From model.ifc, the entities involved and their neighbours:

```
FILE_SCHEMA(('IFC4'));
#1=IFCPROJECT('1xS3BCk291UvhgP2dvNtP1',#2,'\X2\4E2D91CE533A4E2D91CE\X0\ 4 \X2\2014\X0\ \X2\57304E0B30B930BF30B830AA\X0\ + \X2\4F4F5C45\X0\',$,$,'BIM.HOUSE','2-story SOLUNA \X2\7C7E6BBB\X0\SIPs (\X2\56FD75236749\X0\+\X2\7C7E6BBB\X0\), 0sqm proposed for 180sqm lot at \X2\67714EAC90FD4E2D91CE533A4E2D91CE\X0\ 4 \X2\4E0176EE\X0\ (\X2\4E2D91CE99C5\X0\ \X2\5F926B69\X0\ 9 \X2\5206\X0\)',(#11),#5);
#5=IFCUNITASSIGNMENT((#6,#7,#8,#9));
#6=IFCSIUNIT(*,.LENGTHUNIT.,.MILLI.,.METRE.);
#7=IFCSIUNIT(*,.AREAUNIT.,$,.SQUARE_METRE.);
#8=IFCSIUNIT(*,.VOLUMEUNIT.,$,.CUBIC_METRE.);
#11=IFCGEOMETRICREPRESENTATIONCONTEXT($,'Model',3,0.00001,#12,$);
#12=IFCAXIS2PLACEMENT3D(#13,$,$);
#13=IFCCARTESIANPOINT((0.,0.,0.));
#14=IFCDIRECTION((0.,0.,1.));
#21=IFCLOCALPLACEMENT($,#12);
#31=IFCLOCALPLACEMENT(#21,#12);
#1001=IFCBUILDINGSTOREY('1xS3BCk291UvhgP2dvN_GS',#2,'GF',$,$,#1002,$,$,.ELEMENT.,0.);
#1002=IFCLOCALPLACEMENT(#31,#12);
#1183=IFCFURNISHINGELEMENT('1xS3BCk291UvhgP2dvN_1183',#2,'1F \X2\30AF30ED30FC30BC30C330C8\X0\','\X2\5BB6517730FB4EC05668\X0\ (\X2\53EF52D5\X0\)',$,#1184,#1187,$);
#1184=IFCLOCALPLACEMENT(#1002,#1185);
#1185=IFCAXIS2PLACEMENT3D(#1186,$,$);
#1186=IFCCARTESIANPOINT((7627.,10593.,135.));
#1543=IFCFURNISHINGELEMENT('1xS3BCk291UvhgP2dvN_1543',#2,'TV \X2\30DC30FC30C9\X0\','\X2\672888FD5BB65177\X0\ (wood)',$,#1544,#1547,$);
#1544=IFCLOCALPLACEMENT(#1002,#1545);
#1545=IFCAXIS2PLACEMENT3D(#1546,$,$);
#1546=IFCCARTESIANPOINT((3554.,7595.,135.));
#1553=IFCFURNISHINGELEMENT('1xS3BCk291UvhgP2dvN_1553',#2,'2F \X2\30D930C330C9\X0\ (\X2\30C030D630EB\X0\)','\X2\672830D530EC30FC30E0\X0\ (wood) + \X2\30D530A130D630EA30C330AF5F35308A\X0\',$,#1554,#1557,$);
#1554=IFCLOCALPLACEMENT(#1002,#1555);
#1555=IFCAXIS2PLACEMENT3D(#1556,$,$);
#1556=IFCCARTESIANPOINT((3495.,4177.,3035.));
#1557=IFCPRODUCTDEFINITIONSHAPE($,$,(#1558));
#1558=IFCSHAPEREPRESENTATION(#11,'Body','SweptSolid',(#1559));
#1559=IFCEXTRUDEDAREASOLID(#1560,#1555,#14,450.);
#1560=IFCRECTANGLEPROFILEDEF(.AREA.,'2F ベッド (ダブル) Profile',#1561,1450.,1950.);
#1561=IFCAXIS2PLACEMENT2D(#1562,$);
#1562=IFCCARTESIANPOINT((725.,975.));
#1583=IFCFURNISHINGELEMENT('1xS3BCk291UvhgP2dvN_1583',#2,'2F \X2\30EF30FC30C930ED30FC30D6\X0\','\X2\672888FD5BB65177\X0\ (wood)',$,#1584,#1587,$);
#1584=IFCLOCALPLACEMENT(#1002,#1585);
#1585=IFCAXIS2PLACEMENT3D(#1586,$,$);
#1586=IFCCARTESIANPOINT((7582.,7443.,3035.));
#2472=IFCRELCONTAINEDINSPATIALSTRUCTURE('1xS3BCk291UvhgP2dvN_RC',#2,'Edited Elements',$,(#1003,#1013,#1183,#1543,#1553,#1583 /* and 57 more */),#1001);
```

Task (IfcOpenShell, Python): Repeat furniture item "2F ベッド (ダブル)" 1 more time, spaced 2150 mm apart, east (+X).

```python
import numpy as np
import ifcopenshell
import ifcopenshell.api.geometry
import ifcopenshell.api.root
import ifcopenshell.util.element
import ifcopenshell.util.placement
import ifcopenshell.util.unit

model = ifcopenshell.open("model.ifc")
unit_scale = ifcopenshell.util.unit.calculate_unit_scale(model)


def reuse_history(source, copy):
    """copy_class also copies each property set's owner history, people and application; keep the originals."""
    for rel in copy.IsDefinedBy:
        if rel.is_a("IfcRelDefinesByProperties") and (history := rel.RelatingPropertyDefinition.OwnerHistory):
            rel.RelatingPropertyDefinition.OwnerHistory = source.OwnerHistory
            ifcopenshell.util.element.remove_deep2(model, history)


source = model.by_guid("1xS3BCk291UvhgP2dvN_1553")
base = ifcopenshell.util.placement.get_local_placement(source.ObjectPlacement)
step = np.array([1.0, 0.0, 0.0]) * 2.15 / unit_scale

for i in range(1, 2):
    copy = ifcopenshell.api.root.copy_class(model, product=source)
    copy.Representation = ifcopenshell.util.element.copy_deep(
        model, source.Representation, exclude=["IfcGeometricRepresentationContext", "IfcRepresentationMap"]
    )
    reuse_history(source, copy)
    matrix = base.copy()
    matrix[:3, 3] += i * step
    print("added at", matrix[:3, 3].round(3) + 0.0)
    ifcopenshell.api.geometry.edit_object_placement(model, product=copy, matrix=matrix, is_si=False)

model.write("model_edited.ifc")
```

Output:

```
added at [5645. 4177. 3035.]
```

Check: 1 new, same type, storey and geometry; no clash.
